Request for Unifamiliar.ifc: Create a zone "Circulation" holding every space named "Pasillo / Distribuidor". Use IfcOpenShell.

First a look at what the model holds.

```python
import ifcopenshell

model = ifcopenshell.open("Unifamiliar.ifc")
print(model.schema)
seen = {}
for space in model.by_type("IfcSpace"):
    seen[space.LongName] = seen.get(space.LongName, 0) + 1
for name, count in sorted(seen.items(), key=str):
    print(count, "x", name)
print("zones:", [z.Name for z in model.by_type("IfcZone")][:20])
```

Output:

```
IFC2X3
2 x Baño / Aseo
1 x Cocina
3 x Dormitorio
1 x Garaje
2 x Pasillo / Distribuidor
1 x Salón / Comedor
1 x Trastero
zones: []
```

```python
import ifcopenshell
import ifcopenshell.api.group
import ifcopenshell.api.root

model = ifcopenshell.open("Unifamiliar.ifc")

names = {"Pasillo / Distribuidor"}
spaces = [s for s in model.by_type("IfcSpace") if s.LongName in names]

zone = ifcopenshell.api.root.create_entity(model, ifc_class="IfcZone", name="Circulation")
ifcopenshell.api.group.assign_group(model, products=spaces, group=zone)
print(len(spaces), "spaces in", zone.Name)

model.write("Unifamiliar-out.ifc")
```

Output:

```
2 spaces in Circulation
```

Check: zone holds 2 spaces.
